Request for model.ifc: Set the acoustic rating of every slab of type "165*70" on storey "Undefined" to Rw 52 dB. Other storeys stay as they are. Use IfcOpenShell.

First a look at what the model holds.

```python
import ifcopenshell
import ifcopenshell.util.element

model = ifcopenshell.open("model.ifc")
print(model.schema)
storey = next(s for s in model.by_type("IfcBuildingStorey") if s.Name == "Undefined")
slabs = [e for e in ifcopenshell.util.element.get_decomposition(storey) if e.is_a("IfcSlab")]
seen = {}
for e in slabs:
    element_type = ifcopenshell.util.element.get_type(e)
    key = (element_type.Name if element_type != e and element_type else None, ifcopenshell.util.element.get_pset(e, "Pset_SlabCommon", "AcousticRating"))
    seen[key] = seen.get(key, 0) + 1
for (name, value), count in sorted(seen.items(), key=str):
    print(count, "x", name, "|", value)
```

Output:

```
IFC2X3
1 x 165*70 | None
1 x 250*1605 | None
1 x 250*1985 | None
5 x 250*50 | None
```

```python
import ifcopenshell
import ifcopenshell.api.pset
import ifcopenshell.util.element

model = ifcopenshell.open("model.ifc")

storey = next(s for s in model.by_type("IfcBuildingStorey") if s.Name == "Undefined")
slabs = [e for e in ifcopenshell.util.element.get_decomposition(storey) if e.is_a("IfcSlab")]

count = 0
for e in slabs:
    element_type = ifcopenshell.util.element.get_type(e)
    if element_type in (None, e) or element_type.Name != "165*70":
        continue
    # add_pset returns the element's existing set when there is one.
    pset = ifcopenshell.api.pset.add_pset(model, product=e, name="Pset_SlabCommon")
    ifcopenshell.api.pset.edit_pset(model, pset=pset, properties={"AcousticRating": "Rw 52 dB"})
    count += 1

print(count, "slabs updated")

model.write("model_edited.ifc")
```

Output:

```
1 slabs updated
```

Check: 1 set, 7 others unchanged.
